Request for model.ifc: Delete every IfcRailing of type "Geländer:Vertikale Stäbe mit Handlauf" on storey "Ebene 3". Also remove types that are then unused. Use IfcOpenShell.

First a look at what the model holds.

```python
import ifcopenshell
import ifcopenshell.util.element

model = ifcopenshell.open("model.ifc")
print(model.schema)
storey = next(s for s in model.by_type("IfcBuildingStorey") if s.Name == "Ebene 3")
railings = [e for e in ifcopenshell.util.element.get_decomposition(storey) if e.is_a("IfcRailing")]
seen = {}
for e in railings:
    element_type = ifcopenshell.util.element.get_type(e)
    name = element_type.Name if element_type not in (None, e) else None
    seen[name] = seen.get(name, 0) + 1
for name, count in sorted(seen.items(), key=str):
    print(count, "x", name)
```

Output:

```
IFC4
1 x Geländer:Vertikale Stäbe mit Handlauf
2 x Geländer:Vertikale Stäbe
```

```python
import ifcopenshell
import ifcopenshell.api.root
import ifcopenshell.util.element

model = ifcopenshell.open("model.ifc")

storey = next(s for s in model.by_type("IfcBuildingStorey") if s.Name == "Ebene 3")
railings = [e for e in ifcopenshell.util.element.get_decomposition(storey) if e.is_a("IfcRailing")]
targets = [e for e in railings if (t := ifcopenshell.util.element.get_type(e)) not in (None, e) and t.Name == "Geländer:Vertikale Stäbe mit Handlauf"]
types = {ifcopenshell.util.element.get_type(e) for e in targets} - {None, *targets}

for e in targets:
    ifcopenshell.api.root.remove_product(model, product=e)
print(len(targets), "removed")

unused = [t for t in types if not ifcopenshell.util.element.get_types(t)]
for t in unused:
    ifcopenshell.api.root.remove_product(model, product=t)
print(len(unused), "unused types removed")

model.write("model_v2.ifc")
```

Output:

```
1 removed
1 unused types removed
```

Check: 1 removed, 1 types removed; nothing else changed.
